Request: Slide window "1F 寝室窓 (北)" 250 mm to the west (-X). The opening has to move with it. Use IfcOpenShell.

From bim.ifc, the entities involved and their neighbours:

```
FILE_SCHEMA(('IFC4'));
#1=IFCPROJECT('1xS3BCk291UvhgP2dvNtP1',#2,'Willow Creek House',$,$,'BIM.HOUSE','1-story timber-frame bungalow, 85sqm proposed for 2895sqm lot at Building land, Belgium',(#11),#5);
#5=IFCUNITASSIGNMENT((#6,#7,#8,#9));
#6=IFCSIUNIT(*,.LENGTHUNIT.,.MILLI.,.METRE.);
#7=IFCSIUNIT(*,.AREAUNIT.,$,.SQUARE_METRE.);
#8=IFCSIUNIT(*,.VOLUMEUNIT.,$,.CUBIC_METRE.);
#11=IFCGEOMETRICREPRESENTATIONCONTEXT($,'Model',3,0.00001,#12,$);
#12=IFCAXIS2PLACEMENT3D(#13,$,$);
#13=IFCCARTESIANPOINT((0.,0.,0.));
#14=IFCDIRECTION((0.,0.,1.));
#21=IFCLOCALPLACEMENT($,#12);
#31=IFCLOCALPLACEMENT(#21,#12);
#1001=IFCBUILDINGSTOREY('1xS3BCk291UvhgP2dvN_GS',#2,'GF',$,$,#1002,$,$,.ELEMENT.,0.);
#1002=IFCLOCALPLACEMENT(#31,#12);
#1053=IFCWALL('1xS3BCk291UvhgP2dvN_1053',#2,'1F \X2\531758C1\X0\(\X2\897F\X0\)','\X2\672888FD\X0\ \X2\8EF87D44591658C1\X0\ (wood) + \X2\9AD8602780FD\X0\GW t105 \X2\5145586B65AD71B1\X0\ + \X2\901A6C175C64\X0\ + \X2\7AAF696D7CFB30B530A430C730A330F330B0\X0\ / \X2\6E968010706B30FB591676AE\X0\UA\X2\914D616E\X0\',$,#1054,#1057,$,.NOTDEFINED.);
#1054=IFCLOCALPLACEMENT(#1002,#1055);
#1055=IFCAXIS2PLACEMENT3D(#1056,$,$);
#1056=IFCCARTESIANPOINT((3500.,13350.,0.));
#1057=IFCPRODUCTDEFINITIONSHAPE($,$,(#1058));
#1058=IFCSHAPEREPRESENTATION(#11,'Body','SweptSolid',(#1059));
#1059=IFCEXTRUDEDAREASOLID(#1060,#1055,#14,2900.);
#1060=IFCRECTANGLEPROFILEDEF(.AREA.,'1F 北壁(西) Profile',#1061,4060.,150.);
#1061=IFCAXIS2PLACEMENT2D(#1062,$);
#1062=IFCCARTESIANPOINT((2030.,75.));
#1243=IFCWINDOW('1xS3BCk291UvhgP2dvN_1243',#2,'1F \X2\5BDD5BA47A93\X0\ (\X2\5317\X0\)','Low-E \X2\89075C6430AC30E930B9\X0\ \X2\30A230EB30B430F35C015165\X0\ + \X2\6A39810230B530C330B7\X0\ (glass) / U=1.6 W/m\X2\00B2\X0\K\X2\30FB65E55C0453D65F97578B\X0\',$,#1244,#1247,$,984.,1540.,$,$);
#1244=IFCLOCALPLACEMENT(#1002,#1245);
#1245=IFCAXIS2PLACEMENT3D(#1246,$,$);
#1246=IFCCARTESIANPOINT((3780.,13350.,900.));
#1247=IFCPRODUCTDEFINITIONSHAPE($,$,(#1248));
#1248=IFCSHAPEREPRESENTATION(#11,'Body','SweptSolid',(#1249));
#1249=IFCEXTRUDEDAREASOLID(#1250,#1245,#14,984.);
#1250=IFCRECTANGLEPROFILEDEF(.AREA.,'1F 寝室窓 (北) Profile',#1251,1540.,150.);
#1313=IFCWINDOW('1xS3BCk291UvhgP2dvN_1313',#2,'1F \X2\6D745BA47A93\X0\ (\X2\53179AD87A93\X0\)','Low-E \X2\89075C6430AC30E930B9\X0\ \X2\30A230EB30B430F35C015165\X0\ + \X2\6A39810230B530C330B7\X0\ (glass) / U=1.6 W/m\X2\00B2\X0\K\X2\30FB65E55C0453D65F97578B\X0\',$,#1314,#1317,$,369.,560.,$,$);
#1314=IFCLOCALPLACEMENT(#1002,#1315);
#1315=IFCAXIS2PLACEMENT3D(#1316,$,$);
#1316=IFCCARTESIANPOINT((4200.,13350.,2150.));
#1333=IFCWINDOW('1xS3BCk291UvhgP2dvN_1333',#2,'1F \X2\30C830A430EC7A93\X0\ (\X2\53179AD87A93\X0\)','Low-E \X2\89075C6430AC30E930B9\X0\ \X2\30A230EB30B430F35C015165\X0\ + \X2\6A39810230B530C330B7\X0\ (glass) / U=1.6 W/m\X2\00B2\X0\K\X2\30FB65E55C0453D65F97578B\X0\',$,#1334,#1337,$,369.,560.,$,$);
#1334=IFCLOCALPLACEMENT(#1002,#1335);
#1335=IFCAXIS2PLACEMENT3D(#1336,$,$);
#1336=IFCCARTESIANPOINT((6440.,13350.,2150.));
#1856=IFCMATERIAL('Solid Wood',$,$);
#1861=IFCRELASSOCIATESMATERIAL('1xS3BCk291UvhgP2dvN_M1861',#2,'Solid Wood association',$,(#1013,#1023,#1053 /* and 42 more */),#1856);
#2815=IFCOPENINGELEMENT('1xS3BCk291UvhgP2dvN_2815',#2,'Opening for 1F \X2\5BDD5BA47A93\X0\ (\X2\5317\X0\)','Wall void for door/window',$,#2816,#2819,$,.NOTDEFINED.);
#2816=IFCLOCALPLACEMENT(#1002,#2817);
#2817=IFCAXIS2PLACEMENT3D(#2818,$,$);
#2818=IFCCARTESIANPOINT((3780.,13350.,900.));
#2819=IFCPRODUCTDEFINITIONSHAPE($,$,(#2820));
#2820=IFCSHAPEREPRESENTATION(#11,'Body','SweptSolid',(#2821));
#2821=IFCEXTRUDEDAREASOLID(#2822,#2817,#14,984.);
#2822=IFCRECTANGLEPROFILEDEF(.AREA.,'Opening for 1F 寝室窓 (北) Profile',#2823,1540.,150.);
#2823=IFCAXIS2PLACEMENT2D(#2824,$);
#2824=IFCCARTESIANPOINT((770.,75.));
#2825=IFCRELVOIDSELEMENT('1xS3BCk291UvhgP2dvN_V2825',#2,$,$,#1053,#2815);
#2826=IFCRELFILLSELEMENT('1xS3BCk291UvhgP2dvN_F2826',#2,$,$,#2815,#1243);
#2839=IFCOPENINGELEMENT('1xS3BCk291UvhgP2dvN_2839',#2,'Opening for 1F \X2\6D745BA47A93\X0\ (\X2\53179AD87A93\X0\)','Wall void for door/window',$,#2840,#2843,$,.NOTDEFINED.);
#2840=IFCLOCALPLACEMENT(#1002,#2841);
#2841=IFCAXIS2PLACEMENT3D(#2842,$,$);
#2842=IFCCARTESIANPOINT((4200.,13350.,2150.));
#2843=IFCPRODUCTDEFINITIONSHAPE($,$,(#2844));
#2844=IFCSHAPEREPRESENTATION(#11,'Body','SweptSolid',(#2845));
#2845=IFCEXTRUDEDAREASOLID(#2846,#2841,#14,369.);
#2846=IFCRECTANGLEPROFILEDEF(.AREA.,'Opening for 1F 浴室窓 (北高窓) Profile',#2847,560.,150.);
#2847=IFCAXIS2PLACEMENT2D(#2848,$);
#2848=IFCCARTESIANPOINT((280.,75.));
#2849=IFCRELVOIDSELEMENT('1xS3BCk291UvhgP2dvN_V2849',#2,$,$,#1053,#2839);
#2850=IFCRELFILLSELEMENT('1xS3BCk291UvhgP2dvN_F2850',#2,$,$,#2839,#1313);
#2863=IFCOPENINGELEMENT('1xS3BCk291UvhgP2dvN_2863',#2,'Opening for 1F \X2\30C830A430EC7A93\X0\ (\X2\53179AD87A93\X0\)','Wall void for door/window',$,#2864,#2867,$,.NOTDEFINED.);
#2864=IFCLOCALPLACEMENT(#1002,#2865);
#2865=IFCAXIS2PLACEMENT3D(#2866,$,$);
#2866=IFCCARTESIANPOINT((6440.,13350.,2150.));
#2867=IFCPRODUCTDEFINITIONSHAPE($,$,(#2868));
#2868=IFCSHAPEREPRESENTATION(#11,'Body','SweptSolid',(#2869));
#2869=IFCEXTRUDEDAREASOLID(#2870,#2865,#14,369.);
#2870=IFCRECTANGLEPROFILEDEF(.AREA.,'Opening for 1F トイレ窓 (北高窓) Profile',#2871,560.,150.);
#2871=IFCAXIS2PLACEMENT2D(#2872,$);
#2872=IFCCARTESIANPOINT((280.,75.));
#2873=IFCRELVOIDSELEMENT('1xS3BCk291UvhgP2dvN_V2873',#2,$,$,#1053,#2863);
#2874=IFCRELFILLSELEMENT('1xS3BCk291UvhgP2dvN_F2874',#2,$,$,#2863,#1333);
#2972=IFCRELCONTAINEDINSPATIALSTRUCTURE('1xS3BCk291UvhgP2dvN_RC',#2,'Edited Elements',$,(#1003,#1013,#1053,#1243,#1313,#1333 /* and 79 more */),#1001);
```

```python
import ifcopenshell
import ifcopenshell.api.geometry
import ifcopenshell.util.placement
import ifcopenshell.util.unit

model = ifcopenshell.open("bim.ifc")
unit_scale = ifcopenshell.util.unit.calculate_unit_scale(model)

window = model.by_guid("1xS3BCk291UvhgP2dvN_1243")
opening = window.FillsVoids[0].RelatingOpeningElement
wall = opening.VoidsElements[0].RelatingBuildingElement

wall_matrix = ifcopenshell.util.placement.get_local_placement(wall.ObjectPlacement)
shift = wall_matrix[:3, 0] * -0.25 / unit_scale
before = ifcopenshell.util.placement.get_local_placement(window.ObjectPlacement)[:3, 3].copy()

# The window is not placed relative to its opening, so move both.
for product in (opening, window):
    matrix = ifcopenshell.util.placement.get_local_placement(product.ObjectPlacement)
    matrix[:3, 3] += shift
    ifcopenshell.api.geometry.edit_object_placement(model, product=product, matrix=matrix, is_si=False)

after = ifcopenshell.util.placement.get_local_placement(window.ObjectPlacement)[:3, 3]
print("window moved by", (after - before).round(3) + 0.0)

model.write("bim_updated.ifc")
```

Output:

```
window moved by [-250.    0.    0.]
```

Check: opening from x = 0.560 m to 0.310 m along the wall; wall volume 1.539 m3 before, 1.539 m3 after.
